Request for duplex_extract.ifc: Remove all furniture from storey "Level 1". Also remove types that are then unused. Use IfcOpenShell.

First a look at what the model holds.

```python
import ifcopenshell
import ifcopenshell.util.element

model = ifcopenshell.open("duplex_extract.ifc")
print(model.schema)
storey = next(s for s in model.by_type("IfcBuildingStorey") if s.Name == "Level 1")
furniture = [e for e in ifcopenshell.util.element.get_decomposition(storey) if e.is_a("IfcFurnishingElement")]
seen = {}
for e in furniture:
    element_type = ifcopenshell.util.element.get_type(e)
    name = element_type.Name if element_type not in (None, e) else None
    seen[name] = seen.get(name, 0) + 1
for name, count in sorted(seen.items(), key=str):
    print(count, "x", name)
```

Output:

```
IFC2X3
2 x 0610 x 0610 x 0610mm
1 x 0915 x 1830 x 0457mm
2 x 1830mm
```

```python
import ifcopenshell
import ifcopenshell.api.root
import ifcopenshell.util.element

model = ifcopenshell.open("duplex_extract.ifc")

storey = next(s for s in model.by_type("IfcBuildingStorey") if s.Name == "Level 1")
furniture = [e for e in ifcopenshell.util.element.get_decomposition(storey) if e.is_a("IfcFurnishingElement")]
types = {ifcopenshell.util.element.get_type(e) for e in furniture} - {None, *furniture}

for e in furniture:
    ifcopenshell.api.root.remove_product(model, product=e)
print(len(furniture), "removed")

unused = [t for t in types if not ifcopenshell.util.element.get_types(t)]
for t in unused:
    ifcopenshell.api.root.remove_product(model, product=t)
print(len(unused), "unused types removed")

model.write("duplex_extract_edited.ifc")
```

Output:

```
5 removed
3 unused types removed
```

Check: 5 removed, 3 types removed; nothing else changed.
